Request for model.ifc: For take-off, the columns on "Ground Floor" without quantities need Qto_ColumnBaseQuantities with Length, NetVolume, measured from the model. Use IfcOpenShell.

First a look at what the model holds.

```python
import ifcopenshell
import ifcopenshell.util.element
import ifcopenshell.util.unit

model = ifcopenshell.open("model.ifc")
print(model.schema)
for unit_type in ("LENGTHUNIT", "AREAUNIT", "VOLUMEUNIT"):
    print(unit_type, ifcopenshell.util.unit.calculate_unit_scale(model, unit_type))
storey = next(s for s in model.by_type("IfcBuildingStorey") if s.Name == "Ground Floor")
columns = [e for e in ifcopenshell.util.element.get_decomposition(storey) if e.is_a("IfcColumn")]
for e in sorted(columns, key=lambda e: e.id()):
    print(e.id(), e.is_a(), e.Name, list(ifcopenshell.util.element.get_psets(e, qtos_only=True)), sep=" | ")
```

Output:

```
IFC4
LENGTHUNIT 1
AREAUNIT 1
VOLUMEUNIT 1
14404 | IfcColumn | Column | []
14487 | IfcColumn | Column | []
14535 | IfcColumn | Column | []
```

```python
import ifcopenshell
import ifcopenshell.api.pset
import ifcopenshell.geom
import ifcopenshell.util.element
import ifcopenshell.util.shape
import ifcopenshell.util.unit

model = ifcopenshell.open("model.ifc")
unit_scale = ifcopenshell.util.unit.calculate_unit_scale(model)
volume_scale = ifcopenshell.util.unit.calculate_unit_scale(model, "VOLUMEUNIT")
settings = ifcopenshell.geom.settings()

storey = next(s for s in model.by_type("IfcBuildingStorey") if s.Name == "Ground Floor")
columns = [e for e in ifcopenshell.util.element.get_decomposition(storey) if e.is_a("IfcColumn")]

for e in sorted(columns, key=lambda e: e.id()):
    if ifcopenshell.util.element.get_psets(e, qtos_only=True, should_inherit=False):
        continue
    # Geometry comes back in metres, in the element's own axes.
    shape = ifcopenshell.geom.create_shape(settings, e)
    values = {
        "Length": ifcopenshell.util.shape.get_z(shape.geometry) / unit_scale,
        "NetVolume": ifcopenshell.util.shape.get_volume(shape.geometry) / volume_scale,
    }
    qto = ifcopenshell.api.pset.add_qto(model, product=e, name="Qto_ColumnBaseQuantities")
    ifcopenshell.api.pset.edit_qto(model, qto=qto, properties=values)
    print(e.id(), {k: round(v, 3) for k, v in values.items()})

model.write("model_edited.ifc")
```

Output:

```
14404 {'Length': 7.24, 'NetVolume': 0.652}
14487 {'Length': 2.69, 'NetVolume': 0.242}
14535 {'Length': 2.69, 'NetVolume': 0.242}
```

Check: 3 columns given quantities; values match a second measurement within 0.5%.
